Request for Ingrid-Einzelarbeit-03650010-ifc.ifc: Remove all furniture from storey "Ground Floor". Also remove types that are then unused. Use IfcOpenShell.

First a look at what the model holds.

```python
import ifcopenshell
import ifcopenshell.util.element

model = ifcopenshell.open("Ingrid-Einzelarbeit-03650010-ifc.ifc")
print(model.schema)
storey = next(s for s in model.by_type("IfcBuildingStorey") if s.Name == "Ground Floor")
furniture = [e for e in ifcopenshell.util.element.get_decomposition(storey) if e.is_a("IfcFurnishingElement")]
seen = {}
for e in furniture:
    element_type = ifcopenshell.util.element.get_type(e)
    name = element_type.Name if element_type not in (None, e) else None
    seen[name] = seen.get(name, 0) + 1
for name, count in sorted(seen.items(), key=str):
    print(count, "x", name)
```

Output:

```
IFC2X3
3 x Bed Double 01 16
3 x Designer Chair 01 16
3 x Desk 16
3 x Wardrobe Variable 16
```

```python
import ifcopenshell
import ifcopenshell.api.root
import ifcopenshell.util.element

model = ifcopenshell.open("Ingrid-Einzelarbeit-03650010-ifc.ifc")

storey = next(s for s in model.by_type("IfcBuildingStorey") if s.Name == "Ground Floor")
furniture = [e for e in ifcopenshell.util.element.get_decomposition(storey) if e.is_a("IfcFurnishingElement")]
types = {ifcopenshell.util.element.get_type(e) for e in furniture} - {None, *furniture}

for e in furniture:
    ifcopenshell.api.root.remove_product(model, product=e)
print(len(furniture), "removed")

unused = [t for t in types if not ifcopenshell.util.element.get_types(t)]
for t in unused:
    ifcopenshell.api.root.remove_product(model, product=t)
print(len(unused), "unused types removed")

model.write("Ingrid-Einzelarbeit-03650010-ifc-out.ifc")
```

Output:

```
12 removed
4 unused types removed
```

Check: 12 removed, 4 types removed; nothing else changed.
